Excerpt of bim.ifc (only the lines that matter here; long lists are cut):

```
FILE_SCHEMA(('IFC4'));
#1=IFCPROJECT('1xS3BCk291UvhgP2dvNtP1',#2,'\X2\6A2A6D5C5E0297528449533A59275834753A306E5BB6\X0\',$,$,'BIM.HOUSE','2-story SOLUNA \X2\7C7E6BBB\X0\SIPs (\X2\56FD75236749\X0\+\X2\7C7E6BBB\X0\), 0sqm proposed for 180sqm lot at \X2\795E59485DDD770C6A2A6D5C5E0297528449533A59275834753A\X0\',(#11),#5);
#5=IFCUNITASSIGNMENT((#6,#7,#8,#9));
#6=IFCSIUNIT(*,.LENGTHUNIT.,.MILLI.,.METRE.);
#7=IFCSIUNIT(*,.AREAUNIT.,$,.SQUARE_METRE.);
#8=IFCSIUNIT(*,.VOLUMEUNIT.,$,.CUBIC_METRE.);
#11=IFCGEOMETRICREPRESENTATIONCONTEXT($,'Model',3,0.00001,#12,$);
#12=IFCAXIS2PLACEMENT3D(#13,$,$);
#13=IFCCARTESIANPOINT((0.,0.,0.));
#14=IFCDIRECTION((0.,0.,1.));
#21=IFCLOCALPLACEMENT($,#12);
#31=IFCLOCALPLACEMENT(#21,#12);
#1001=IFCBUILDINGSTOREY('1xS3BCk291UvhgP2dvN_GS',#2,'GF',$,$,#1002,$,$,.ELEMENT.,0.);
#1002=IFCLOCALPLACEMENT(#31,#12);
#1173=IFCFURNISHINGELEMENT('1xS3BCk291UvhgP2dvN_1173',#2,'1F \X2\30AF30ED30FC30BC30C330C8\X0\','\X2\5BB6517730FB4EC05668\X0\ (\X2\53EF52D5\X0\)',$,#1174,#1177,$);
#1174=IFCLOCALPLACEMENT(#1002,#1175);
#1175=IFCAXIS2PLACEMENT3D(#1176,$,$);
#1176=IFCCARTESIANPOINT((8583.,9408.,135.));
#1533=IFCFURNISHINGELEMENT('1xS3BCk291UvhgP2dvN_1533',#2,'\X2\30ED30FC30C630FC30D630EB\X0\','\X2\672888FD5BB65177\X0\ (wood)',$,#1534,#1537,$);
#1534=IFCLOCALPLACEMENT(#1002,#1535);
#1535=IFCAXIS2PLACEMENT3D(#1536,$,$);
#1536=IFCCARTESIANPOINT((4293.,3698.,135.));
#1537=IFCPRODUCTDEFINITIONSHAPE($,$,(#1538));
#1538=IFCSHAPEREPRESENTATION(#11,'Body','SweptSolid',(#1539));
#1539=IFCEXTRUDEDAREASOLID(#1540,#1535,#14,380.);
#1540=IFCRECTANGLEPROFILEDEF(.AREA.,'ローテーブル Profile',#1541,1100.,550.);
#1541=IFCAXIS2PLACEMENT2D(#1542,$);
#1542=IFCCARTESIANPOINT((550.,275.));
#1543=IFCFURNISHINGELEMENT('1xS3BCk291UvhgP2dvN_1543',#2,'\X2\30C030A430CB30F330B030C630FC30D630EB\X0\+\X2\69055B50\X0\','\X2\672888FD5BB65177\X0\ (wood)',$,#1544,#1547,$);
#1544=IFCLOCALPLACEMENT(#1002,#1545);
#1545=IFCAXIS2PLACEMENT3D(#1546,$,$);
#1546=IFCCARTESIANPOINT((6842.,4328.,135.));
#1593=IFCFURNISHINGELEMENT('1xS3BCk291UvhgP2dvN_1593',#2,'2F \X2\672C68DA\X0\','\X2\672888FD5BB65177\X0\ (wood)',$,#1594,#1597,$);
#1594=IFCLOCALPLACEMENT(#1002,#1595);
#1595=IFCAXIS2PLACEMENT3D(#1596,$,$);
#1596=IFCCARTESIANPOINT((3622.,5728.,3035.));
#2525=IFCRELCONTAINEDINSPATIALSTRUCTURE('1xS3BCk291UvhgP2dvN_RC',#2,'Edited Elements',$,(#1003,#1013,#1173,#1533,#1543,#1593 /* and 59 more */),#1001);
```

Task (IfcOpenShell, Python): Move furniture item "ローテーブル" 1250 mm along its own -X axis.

```python
import ifcopenshell
import ifcopenshell.api.geometry
import ifcopenshell.util.placement
import ifcopenshell.util.unit

model = ifcopenshell.open("bim.ifc")
unit_scale = ifcopenshell.util.unit.calculate_unit_scale(model)

item = model.by_guid("1xS3BCk291UvhgP2dvN_1533")
matrix = ifcopenshell.util.placement.get_local_placement(item.ObjectPlacement)
matrix[:3, 3] -= matrix[:3, 0] * 1.25 / unit_scale
ifcopenshell.api.geometry.edit_object_placement(model, product=item, matrix=matrix, is_si=False)

print(ifcopenshell.util.placement.get_local_placement(item.ObjectPlacement).round(3) + 0.0)

model.write("bim-out.ifc")
```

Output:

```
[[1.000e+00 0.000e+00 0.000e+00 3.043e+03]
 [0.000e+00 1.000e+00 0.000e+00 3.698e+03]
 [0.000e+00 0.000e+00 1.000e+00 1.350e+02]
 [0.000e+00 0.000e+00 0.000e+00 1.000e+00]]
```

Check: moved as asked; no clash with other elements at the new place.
